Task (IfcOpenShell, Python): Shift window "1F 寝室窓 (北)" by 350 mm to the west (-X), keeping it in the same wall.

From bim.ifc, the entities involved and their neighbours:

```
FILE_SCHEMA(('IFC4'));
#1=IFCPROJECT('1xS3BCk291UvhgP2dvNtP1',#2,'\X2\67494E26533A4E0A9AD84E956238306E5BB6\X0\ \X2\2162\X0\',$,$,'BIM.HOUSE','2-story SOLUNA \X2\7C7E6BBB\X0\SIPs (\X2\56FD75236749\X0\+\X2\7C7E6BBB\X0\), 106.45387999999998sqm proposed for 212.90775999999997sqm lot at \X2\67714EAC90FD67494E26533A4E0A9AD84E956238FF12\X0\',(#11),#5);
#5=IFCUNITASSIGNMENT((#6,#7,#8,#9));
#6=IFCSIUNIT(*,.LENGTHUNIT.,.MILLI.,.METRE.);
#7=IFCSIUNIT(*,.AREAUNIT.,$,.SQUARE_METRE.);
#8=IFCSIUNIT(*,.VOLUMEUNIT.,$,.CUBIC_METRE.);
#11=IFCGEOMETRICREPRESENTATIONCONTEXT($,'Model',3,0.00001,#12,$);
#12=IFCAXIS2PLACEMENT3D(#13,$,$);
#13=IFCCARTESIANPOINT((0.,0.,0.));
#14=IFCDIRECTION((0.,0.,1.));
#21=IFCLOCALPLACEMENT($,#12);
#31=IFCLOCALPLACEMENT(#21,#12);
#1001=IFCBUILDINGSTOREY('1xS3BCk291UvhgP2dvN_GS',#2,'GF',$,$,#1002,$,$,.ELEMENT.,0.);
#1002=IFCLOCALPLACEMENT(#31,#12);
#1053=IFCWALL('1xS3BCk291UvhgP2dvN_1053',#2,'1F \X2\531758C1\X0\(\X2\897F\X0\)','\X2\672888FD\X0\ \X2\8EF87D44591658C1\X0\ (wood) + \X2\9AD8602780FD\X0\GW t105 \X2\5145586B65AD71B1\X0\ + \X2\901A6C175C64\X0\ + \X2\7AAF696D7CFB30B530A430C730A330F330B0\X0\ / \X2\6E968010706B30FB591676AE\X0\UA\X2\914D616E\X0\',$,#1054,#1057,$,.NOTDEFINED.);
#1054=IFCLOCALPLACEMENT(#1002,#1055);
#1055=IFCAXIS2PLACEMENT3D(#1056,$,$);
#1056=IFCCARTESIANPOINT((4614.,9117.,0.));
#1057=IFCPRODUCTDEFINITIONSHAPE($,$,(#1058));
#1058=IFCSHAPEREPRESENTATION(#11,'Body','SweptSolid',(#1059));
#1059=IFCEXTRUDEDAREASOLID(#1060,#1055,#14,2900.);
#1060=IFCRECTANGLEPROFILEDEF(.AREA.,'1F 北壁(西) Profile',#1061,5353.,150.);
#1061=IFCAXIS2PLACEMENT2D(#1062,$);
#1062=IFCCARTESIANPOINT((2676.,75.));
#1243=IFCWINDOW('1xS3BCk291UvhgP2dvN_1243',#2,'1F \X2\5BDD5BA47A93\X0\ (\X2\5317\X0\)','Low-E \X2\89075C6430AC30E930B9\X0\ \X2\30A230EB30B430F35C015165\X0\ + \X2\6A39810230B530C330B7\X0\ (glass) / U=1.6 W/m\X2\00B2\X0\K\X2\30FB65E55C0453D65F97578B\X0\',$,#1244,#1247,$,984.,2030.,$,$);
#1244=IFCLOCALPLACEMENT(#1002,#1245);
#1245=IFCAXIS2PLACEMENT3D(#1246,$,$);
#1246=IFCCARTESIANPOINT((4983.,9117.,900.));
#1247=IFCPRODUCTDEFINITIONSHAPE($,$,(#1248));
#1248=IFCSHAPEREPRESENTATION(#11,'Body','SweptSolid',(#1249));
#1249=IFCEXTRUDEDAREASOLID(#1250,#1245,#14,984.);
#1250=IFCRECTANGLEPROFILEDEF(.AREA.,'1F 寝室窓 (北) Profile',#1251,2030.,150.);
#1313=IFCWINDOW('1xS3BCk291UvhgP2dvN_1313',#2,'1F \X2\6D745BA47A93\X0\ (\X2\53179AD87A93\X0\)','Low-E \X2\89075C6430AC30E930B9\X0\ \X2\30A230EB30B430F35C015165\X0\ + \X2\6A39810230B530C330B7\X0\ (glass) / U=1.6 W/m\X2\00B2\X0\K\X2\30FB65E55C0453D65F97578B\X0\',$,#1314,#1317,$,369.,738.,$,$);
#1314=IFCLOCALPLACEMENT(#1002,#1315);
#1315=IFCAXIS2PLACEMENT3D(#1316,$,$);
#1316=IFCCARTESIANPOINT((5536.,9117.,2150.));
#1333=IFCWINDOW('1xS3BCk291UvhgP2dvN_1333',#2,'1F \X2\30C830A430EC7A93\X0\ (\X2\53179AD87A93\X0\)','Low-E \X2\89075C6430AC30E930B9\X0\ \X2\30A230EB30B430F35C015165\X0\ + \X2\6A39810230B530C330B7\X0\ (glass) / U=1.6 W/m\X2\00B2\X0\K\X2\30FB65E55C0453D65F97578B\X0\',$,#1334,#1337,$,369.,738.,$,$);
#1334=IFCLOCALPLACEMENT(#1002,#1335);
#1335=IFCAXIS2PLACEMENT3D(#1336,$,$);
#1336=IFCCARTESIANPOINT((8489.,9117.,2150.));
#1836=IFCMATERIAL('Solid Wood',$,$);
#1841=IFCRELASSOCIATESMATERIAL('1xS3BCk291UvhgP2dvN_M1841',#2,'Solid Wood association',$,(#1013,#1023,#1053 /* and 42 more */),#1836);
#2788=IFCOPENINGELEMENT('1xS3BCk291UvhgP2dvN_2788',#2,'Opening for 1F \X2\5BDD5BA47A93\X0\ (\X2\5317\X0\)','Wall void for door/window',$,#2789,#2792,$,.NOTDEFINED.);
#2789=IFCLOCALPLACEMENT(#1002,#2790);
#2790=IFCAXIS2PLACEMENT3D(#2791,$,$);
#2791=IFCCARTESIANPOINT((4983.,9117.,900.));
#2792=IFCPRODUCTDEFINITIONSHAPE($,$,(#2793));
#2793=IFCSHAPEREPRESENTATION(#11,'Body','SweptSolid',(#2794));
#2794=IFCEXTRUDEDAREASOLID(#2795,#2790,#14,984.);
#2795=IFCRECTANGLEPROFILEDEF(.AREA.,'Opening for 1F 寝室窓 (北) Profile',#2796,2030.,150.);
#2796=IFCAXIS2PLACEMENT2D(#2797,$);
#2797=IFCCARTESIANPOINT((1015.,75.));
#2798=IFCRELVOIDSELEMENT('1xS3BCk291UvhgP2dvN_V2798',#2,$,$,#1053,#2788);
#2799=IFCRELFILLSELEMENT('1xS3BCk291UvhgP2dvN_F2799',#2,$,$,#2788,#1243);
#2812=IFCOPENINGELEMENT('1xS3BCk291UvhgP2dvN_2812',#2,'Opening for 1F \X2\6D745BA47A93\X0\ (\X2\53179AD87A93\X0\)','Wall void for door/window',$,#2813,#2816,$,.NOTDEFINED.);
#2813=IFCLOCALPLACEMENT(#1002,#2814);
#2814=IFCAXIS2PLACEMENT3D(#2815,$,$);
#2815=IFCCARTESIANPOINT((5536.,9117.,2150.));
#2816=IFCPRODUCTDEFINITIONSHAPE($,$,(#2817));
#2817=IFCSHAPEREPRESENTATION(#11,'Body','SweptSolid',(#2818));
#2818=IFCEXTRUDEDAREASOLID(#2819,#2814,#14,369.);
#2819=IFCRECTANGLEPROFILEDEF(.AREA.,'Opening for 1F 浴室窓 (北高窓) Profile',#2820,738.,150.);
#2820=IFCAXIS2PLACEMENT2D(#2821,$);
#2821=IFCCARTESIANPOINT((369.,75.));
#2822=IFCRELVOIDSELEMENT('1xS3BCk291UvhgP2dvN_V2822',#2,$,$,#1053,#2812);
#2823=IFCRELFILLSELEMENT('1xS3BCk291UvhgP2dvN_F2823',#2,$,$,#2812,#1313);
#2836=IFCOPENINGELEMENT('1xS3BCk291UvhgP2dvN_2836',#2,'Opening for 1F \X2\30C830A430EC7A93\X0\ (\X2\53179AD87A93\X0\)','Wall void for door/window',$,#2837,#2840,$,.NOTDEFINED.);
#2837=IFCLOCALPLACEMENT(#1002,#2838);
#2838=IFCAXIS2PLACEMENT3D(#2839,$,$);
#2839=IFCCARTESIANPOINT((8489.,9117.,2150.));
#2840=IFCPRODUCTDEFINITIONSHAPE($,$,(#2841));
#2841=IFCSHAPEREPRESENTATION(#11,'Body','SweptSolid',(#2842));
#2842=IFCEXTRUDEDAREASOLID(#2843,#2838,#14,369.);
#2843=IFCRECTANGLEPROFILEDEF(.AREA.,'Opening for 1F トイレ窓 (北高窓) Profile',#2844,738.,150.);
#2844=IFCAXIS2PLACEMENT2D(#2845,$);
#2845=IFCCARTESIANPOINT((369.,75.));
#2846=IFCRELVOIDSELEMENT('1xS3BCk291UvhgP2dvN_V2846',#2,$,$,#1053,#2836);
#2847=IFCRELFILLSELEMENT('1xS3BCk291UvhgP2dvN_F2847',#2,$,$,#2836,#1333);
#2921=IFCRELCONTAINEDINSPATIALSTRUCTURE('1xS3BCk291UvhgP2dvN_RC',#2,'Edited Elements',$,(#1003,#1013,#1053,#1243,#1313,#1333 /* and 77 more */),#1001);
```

```python
import ifcopenshell
import ifcopenshell.api.geometry
import ifcopenshell.util.placement

model = ifcopenshell.open("bim.ifc")

window = model.by_guid("1xS3BCk291UvhgP2dvN_1243")
opening = window.FillsVoids[0].RelatingOpeningElement
wall = opening.VoidsElements[0].RelatingBuildingElement

wall_matrix = ifcopenshell.util.placement.get_local_placement(wall.ObjectPlacement)
shift = wall_matrix[:3, 0] * -350.0
before = ifcopenshell.util.placement.get_local_placement(window.ObjectPlacement)[:3, 3].copy()

# The window is not placed relative to its opening, so move both.
for product in (opening, window):
    matrix = ifcopenshell.util.placement.get_local_placement(product.ObjectPlacement)
    matrix[:3, 3] += shift
    ifcopenshell.api.geometry.edit_object_placement(model, product=product, matrix=matrix, is_si=False)

after = ifcopenshell.util.placement.get_local_placement(window.ObjectPlacement)[:3, 3]
print("window moved by", (after - before).round(3) + 0.0)

model.write("bim_v2.ifc")
```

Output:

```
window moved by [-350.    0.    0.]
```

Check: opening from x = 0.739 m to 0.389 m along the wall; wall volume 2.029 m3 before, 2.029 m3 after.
